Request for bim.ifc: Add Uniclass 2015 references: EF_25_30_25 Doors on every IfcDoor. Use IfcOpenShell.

First a look at what the model holds.

```python
import ifcopenshell

model = ifcopenshell.open("bim.ifc")
print(model.schema)
print("classifications:", [c.Name for c in model.by_type("IfcClassification")])
for ifc_class in ("IfcDoor", "IfcRoof", "IfcStair", "IfcWall", "IfcWindow"):
    print(ifc_class, len(model.by_type(ifc_class)))
```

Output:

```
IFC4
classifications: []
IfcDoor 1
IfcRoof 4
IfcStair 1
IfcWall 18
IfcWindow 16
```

```python
import ifcopenshell
import ifcopenshell.api.classification

model = ifcopenshell.open("bim.ifc")

system = ifcopenshell.api.classification.add_classification(model, classification="Uniclass 2015")

codes = {
    "IfcDoor": ("EF_25_30_25", "Doors"),
}
for ifc_class, (code, name) in codes.items():
    products = model.by_type(ifc_class)
    ifcopenshell.api.classification.add_reference(
        model, products=products, classification=system, identification=code, name=name
    )
    print(code, len(products))

model.write("bim-out.ifc")
```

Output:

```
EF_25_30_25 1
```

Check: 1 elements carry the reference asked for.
